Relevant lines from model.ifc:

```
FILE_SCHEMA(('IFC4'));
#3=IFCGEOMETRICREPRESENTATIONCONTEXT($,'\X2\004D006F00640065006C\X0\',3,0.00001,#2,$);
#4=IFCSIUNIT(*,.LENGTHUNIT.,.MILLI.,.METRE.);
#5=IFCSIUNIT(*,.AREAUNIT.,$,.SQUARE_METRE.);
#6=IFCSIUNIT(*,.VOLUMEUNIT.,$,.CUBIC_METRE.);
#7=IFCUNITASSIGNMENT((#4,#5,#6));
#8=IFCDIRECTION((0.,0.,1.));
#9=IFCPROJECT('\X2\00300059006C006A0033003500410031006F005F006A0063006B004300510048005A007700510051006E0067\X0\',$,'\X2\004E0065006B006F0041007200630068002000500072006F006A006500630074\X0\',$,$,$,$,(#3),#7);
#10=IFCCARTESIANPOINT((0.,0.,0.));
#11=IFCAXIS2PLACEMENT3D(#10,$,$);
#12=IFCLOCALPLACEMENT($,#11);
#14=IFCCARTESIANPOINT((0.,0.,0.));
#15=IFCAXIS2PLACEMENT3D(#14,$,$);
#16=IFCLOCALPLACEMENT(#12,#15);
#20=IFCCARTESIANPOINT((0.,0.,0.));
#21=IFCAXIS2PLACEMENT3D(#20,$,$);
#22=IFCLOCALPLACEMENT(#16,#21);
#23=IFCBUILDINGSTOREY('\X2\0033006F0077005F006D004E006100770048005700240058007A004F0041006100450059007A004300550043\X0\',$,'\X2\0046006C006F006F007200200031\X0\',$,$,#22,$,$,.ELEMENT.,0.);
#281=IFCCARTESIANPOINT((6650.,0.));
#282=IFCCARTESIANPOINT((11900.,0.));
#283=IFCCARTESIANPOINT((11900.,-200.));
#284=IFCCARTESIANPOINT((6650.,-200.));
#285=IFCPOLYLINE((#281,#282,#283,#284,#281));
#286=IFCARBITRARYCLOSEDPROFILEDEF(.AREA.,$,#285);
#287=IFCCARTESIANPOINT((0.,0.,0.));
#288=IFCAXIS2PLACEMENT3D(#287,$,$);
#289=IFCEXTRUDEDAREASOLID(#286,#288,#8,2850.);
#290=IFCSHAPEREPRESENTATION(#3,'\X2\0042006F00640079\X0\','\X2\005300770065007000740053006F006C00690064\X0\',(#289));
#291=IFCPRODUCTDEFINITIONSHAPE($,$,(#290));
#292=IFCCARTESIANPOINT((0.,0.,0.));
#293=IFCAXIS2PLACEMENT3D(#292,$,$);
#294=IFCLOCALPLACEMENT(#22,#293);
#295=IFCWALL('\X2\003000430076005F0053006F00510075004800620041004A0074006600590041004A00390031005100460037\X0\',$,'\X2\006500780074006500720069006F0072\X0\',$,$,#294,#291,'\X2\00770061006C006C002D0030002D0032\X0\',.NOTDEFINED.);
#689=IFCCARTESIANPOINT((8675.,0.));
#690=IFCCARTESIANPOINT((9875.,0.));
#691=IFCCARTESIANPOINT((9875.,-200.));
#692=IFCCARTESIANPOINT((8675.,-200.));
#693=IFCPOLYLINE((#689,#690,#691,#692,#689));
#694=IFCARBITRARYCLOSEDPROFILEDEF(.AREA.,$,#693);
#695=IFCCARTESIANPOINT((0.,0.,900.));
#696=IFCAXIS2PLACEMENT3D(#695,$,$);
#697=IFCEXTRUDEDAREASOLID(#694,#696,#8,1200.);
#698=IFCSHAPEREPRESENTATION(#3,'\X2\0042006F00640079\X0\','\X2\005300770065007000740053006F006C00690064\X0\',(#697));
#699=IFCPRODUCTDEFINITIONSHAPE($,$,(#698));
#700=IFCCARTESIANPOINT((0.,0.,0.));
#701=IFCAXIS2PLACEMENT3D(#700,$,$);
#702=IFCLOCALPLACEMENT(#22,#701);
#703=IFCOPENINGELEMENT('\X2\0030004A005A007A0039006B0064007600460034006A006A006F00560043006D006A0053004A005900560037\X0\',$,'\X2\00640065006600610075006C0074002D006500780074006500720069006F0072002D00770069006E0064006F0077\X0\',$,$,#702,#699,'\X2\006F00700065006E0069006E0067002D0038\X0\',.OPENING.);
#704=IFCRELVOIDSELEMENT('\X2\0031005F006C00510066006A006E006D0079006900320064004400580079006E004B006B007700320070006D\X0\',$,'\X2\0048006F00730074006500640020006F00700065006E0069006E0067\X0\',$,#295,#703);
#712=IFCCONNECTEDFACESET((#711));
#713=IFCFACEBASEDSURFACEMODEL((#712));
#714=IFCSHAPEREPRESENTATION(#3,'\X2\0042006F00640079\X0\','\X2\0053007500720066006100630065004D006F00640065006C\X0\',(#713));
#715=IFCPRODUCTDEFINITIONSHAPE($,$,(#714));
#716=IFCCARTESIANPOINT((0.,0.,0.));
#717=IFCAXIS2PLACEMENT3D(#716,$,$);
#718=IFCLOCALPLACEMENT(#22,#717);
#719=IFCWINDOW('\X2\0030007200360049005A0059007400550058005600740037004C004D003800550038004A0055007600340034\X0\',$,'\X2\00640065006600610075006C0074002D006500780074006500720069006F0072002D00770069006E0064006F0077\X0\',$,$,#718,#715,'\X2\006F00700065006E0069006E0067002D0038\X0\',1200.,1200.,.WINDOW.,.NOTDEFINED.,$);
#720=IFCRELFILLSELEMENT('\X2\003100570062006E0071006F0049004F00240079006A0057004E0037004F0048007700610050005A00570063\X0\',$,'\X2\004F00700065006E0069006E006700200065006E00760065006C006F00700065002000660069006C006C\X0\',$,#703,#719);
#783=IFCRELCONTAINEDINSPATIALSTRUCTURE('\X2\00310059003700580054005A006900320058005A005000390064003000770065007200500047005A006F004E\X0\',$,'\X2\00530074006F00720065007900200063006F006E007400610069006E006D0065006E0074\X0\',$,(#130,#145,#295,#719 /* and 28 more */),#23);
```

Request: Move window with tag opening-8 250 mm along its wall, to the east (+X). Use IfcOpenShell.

```python
import ifcopenshell
import ifcopenshell.api.geometry
import ifcopenshell.util.placement

model = ifcopenshell.open("model.ifc")

window = model.by_id(719)
opening = window.FillsVoids[0].RelatingOpeningElement
wall = opening.VoidsElements[0].RelatingBuildingElement

wall_matrix = ifcopenshell.util.placement.get_local_placement(wall.ObjectPlacement)
shift = wall_matrix[:3, 0] * 250.0
before = ifcopenshell.util.placement.get_local_placement(window.ObjectPlacement)[:3, 3].copy()

# The window is not placed relative to its opening, so move both.
for product in (opening, window):
    matrix = ifcopenshell.util.placement.get_local_placement(product.ObjectPlacement)
    matrix[:3, 3] += shift
    ifcopenshell.api.geometry.edit_object_placement(model, product=product, matrix=matrix, is_si=False)

after = ifcopenshell.util.placement.get_local_placement(window.ObjectPlacement)[:3, 3]
print("window moved by", (after - before).round(3) + 0.0)

model.write("model_rev.ifc")
```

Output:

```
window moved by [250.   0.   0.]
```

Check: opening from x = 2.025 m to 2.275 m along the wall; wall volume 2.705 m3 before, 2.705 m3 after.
